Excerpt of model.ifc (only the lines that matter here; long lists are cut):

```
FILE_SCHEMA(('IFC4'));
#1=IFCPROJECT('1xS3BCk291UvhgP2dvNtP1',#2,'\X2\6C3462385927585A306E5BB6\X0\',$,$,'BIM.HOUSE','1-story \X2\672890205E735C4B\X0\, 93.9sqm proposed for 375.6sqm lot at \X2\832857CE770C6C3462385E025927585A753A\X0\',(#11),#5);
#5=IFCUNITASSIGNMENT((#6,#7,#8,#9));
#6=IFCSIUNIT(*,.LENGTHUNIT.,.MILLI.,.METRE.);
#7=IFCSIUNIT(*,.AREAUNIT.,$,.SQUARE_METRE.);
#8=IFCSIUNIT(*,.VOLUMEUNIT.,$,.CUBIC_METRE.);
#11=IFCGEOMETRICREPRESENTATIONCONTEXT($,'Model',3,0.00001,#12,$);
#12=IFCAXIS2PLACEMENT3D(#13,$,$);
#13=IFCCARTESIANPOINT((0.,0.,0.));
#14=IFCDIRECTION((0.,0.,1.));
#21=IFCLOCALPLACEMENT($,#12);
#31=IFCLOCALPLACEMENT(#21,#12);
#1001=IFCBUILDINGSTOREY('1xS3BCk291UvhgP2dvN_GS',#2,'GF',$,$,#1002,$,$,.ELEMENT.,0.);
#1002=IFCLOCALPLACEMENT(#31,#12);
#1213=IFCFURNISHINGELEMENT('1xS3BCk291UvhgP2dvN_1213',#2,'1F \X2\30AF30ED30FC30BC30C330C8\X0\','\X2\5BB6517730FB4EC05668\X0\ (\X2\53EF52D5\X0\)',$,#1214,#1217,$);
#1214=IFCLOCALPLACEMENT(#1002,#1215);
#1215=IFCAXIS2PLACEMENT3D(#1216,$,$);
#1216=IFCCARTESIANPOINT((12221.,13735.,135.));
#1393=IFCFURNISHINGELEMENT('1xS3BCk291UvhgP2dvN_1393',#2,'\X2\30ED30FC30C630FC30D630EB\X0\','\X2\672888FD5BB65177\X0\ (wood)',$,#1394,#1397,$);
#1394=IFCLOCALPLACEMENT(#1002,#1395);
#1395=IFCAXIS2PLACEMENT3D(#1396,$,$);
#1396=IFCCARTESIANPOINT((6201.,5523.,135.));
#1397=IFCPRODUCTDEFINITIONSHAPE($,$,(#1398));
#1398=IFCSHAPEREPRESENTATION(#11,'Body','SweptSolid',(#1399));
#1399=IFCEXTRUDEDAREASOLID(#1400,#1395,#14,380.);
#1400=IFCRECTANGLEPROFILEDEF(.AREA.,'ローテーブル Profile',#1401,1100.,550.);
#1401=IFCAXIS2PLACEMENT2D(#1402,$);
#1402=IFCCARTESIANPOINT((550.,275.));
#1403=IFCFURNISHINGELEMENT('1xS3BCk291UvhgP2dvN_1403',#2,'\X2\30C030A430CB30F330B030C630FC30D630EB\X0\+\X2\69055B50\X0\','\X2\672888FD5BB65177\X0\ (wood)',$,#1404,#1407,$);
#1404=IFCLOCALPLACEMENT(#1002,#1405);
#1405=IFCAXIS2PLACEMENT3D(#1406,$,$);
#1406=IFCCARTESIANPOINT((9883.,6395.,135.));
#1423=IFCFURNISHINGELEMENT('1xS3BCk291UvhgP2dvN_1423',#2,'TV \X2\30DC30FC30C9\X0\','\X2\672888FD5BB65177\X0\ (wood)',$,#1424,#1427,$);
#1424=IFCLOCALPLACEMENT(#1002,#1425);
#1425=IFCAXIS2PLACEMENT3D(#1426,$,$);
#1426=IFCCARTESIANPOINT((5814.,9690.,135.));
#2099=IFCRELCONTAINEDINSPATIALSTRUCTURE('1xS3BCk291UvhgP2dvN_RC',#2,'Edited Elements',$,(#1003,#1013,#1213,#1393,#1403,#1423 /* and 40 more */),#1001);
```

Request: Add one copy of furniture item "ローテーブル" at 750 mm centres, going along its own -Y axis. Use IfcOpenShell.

```python
import ifcopenshell
import ifcopenshell.api.geometry
import ifcopenshell.api.root
import ifcopenshell.util.element
import ifcopenshell.util.placement
import ifcopenshell.util.unit

model = ifcopenshell.open("model.ifc")
unit_scale = ifcopenshell.util.unit.calculate_unit_scale(model)


def reuse_history(source, copy):
    """copy_class also copies each property set's owner history, people and application; keep the originals."""
    for rel in copy.IsDefinedBy:
        if rel.is_a("IfcRelDefinesByProperties") and (history := rel.RelatingPropertyDefinition.OwnerHistory):
            rel.RelatingPropertyDefinition.OwnerHistory = source.OwnerHistory
            ifcopenshell.util.element.remove_deep2(model, history)


source = model.by_id(1393)
base = ifcopenshell.util.placement.get_local_placement(source.ObjectPlacement)
step = -base[:3, 1] * 0.75 / unit_scale

for i in range(1, 2):
    copy = ifcopenshell.api.root.copy_class(model, product=source)
    copy.Representation = ifcopenshell.util.element.copy_deep(
        model, source.Representation, exclude=["IfcGeometricRepresentationContext", "IfcRepresentationMap"]
    )
    reuse_history(source, copy)
    matrix = base.copy()
    matrix[:3, 3] += i * step
    print("added at", matrix[:3, 3].round(3) + 0.0)
    ifcopenshell.api.geometry.edit_object_placement(model, product=copy, matrix=matrix, is_si=False)

model.write("model_rev.ifc")
```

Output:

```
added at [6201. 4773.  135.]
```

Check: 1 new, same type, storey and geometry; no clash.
